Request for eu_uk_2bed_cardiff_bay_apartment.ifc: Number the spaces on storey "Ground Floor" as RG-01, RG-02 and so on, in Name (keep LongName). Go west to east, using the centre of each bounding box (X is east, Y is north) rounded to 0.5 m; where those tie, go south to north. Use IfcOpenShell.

First a look at what the model holds.

```python
import ifcopenshell
import ifcopenshell.util.element
import ifcopenshell.util.placement

model = ifcopenshell.open("eu_uk_2bed_cardiff_bay_apartment.ifc")
print(model.schema)
storey = next(s for s in model.by_type("IfcBuildingStorey") if s.Name == "Ground Floor")
spaces = [e for e in ifcopenshell.util.element.get_decomposition(storey) if e.is_a("IfcSpace")]
for e in sorted(spaces, key=lambda e: e.id()):
    origin = ifcopenshell.util.placement.get_local_placement(e.ObjectPlacement)[:3, 3]
    print(e.id(), e.Name, e.LongName, origin.round(2) + 0.0, sep=" | ")
```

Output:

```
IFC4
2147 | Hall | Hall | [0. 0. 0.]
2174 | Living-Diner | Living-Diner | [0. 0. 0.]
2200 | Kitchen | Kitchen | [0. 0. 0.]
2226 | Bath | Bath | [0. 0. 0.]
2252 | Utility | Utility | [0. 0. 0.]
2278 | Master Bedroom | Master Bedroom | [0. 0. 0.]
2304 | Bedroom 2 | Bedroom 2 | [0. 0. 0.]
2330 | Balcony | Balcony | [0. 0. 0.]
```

```python
import ifcopenshell
import ifcopenshell.geom
import ifcopenshell.util.element
import ifcopenshell.util.shape

model = ifcopenshell.open("eu_uk_2bed_cardiff_bay_apartment.ifc")
settings = ifcopenshell.geom.settings()
settings.set("use-world-coords", True)


def centre(element):
    shape = ifcopenshell.geom.create_shape(settings, element)
    return ifcopenshell.util.shape.get_bbox_centroid(shape.geometry)


storey = next(s for s in model.by_type("IfcBuildingStorey") if s.Name == "Ground Floor")
spaces = [e for e in ifcopenshell.util.element.get_decomposition(storey) if e.is_a("IfcSpace")]

# Insertion points can sit at a corner or the storey origin, so sort by the geometry (in metres).
centres = {e: centre(e) for e in spaces}
spaces.sort(key=lambda e: (round(centres[e][0] / 0.5), centres[e][1]))

for i, e in enumerate(spaces, start=1):
    number = f"RG-{i:02d}"
    e.Name = number
    print(e.id(), number)

model.write("eu_uk_2bed_cardiff_bay_apartment_v2.ifc")
```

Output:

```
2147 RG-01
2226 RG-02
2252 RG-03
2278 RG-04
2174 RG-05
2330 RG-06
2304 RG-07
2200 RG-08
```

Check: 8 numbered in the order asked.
